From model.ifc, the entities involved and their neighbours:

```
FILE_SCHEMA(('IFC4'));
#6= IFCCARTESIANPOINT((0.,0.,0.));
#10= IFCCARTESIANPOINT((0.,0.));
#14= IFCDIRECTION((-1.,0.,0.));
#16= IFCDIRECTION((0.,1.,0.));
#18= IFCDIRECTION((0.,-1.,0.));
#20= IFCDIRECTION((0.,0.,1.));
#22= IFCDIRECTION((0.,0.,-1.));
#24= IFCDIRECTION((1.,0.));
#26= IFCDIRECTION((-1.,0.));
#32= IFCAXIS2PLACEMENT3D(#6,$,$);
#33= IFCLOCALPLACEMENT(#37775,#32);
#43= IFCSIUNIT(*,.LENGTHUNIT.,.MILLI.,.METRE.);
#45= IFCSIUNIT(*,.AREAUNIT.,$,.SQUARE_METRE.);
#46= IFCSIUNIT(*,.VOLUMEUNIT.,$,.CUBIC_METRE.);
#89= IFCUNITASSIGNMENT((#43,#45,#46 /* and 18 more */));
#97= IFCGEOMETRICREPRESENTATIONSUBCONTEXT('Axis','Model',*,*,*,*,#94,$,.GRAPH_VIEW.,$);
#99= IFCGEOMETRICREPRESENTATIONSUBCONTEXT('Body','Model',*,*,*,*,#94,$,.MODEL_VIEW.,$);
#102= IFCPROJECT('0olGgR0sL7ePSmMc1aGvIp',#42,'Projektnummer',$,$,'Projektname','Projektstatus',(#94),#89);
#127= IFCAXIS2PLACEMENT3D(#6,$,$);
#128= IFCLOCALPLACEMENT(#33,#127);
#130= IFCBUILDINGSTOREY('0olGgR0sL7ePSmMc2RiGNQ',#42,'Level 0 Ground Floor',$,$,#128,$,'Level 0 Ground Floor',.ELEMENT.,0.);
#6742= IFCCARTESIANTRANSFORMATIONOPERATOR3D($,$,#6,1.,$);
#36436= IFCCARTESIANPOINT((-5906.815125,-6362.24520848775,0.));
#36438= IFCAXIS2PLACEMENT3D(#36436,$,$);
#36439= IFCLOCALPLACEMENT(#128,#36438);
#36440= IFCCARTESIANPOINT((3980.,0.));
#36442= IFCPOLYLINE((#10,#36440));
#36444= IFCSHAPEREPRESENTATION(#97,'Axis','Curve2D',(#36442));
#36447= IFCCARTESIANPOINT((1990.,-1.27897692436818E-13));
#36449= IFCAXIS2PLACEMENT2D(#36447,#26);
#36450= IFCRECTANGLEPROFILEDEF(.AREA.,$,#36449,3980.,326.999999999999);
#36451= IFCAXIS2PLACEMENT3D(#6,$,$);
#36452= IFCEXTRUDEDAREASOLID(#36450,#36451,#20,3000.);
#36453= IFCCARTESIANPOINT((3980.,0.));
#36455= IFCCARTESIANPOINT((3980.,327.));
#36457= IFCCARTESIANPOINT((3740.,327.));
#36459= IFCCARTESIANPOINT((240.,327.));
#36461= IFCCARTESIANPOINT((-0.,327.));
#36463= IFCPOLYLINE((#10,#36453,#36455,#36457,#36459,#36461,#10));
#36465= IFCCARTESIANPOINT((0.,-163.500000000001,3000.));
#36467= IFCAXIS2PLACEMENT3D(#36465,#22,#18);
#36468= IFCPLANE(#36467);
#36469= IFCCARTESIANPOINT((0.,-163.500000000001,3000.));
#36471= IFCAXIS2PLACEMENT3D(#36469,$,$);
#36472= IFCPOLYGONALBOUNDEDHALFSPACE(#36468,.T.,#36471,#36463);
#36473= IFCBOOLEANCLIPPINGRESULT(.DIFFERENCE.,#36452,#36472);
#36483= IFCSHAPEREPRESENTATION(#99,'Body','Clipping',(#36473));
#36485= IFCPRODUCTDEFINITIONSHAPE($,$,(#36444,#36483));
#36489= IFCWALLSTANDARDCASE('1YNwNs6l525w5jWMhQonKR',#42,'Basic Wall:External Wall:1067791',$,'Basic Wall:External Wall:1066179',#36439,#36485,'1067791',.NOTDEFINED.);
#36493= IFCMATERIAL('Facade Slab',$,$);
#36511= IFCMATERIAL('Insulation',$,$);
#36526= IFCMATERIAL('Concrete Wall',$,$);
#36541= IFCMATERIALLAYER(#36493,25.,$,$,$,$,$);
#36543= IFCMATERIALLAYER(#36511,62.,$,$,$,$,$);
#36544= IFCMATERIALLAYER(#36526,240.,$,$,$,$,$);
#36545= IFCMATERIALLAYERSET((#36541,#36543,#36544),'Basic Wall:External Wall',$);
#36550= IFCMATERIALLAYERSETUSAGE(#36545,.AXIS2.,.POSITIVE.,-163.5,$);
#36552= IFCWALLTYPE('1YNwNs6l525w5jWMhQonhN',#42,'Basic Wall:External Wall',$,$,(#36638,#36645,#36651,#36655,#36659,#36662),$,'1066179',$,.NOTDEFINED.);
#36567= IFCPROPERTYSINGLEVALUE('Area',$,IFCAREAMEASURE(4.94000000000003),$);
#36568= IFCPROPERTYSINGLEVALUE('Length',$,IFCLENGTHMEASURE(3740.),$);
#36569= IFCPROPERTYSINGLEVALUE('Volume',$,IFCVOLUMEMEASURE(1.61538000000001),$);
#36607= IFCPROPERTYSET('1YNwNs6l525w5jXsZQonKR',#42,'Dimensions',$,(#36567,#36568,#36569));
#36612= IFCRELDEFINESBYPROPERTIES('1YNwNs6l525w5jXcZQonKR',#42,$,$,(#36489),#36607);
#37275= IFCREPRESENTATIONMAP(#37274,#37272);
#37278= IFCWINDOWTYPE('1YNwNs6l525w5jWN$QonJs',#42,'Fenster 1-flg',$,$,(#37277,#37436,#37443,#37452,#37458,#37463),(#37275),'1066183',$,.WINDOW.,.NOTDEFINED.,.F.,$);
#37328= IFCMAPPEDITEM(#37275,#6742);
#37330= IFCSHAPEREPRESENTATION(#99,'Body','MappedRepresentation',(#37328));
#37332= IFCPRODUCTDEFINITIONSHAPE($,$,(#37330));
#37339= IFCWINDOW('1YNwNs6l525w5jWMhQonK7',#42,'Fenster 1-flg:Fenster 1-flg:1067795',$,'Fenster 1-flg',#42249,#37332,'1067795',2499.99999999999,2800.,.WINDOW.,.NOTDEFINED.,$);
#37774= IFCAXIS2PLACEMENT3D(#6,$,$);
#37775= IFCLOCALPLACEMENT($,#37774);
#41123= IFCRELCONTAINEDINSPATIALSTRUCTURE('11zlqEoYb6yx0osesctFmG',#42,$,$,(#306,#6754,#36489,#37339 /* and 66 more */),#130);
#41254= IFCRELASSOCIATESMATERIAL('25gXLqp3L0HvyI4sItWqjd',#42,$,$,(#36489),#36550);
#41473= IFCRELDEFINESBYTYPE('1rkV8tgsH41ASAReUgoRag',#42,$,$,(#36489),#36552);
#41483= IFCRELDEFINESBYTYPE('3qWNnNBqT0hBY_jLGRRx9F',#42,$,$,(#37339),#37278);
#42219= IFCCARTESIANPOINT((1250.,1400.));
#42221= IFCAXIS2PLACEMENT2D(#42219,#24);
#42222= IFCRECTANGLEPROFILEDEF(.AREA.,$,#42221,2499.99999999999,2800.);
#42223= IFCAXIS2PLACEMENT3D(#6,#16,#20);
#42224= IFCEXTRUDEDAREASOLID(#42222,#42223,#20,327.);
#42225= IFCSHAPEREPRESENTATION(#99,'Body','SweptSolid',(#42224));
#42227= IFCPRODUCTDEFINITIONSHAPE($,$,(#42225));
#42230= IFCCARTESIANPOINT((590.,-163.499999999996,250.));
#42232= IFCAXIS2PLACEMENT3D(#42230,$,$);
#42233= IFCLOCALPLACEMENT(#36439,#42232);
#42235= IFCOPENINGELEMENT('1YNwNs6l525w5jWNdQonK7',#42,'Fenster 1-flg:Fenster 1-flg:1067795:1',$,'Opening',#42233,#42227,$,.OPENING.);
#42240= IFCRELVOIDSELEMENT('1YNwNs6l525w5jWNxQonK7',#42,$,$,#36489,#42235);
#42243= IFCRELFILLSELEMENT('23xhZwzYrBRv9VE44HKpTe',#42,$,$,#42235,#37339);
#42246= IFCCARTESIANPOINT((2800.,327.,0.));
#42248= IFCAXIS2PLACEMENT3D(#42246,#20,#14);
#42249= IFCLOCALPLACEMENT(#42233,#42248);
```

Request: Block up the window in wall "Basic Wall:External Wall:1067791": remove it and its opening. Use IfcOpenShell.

```python
import ifcopenshell
import ifcopenshell.api.feature
import ifcopenshell.api.pset
import ifcopenshell.api.root
import ifcopenshell.geom
import ifcopenshell.util.element
import ifcopenshell.util.shape
import ifcopenshell.util.unit

model = ifcopenshell.open("model.ifc")
area_scale = ifcopenshell.util.unit.calculate_unit_scale(model, "AREAUNIT")
volume_scale = ifcopenshell.util.unit.calculate_unit_scale(model, "VOLUMEUNIT")
settings = ifcopenshell.geom.settings()


def volume(element):
    """Net volume in cubic metres, openings subtracted."""
    shape = ifcopenshell.geom.create_shape(settings, element)
    return ifcopenshell.util.shape.get_volume(shape.geometry)


window = model.by_guid("1YNwNs6l525w5jWMhQonK7")
opening = window.FillsVoids[0].RelatingOpeningElement
wall = opening.VoidsElements[0].RelatingBuildingElement
before = volume(wall)

ifcopenshell.api.root.remove_product(model, product=window)
ifcopenshell.api.feature.remove_feature(model, feature=opening)

after = volume(wall)
thickness = 0.327  # wall thickness in metres

# Update the wall's stored quantities.
pset = model.by_id(ifcopenshell.util.element.get_pset(wall, "Dimensions", should_inherit=False)["id"])
ifcopenshell.api.pset.edit_pset(model, pset=pset, properties={
    "Area": model.create_entity("IfcAreaMeasure", after / thickness / area_scale),
    "Volume": model.create_entity("IfcVolumeMeasure", after / volume_scale),
})

print(f"wall volume {before:.3f} -> {after:.3f} m3")

model.write("model_rev.ifc")
```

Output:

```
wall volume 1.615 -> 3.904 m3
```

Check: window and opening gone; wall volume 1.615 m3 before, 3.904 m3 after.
